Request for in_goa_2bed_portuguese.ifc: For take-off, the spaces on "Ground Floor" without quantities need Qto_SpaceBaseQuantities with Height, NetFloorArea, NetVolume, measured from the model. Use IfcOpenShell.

First a look at what the model holds.

```python
import ifcopenshell
import ifcopenshell.util.element
import ifcopenshell.util.unit

model = ifcopenshell.open("in_goa_2bed_portuguese.ifc")
print(model.schema)
for unit_type in ("LENGTHUNIT", "AREAUNIT", "VOLUMEUNIT"):
    print(unit_type, ifcopenshell.util.unit.calculate_unit_scale(model, unit_type))
storey = next(s for s in model.by_type("IfcBuildingStorey") if s.Name == "Ground Floor")
spaces = [e for e in ifcopenshell.util.element.get_decomposition(storey) if e.is_a("IfcSpace")]
for e in sorted(spaces, key=lambda e: e.id()):
    print(e.id(), e.is_a(), e.Name, list(ifcopenshell.util.element.get_psets(e, qtos_only=True)), sep=" | ")
```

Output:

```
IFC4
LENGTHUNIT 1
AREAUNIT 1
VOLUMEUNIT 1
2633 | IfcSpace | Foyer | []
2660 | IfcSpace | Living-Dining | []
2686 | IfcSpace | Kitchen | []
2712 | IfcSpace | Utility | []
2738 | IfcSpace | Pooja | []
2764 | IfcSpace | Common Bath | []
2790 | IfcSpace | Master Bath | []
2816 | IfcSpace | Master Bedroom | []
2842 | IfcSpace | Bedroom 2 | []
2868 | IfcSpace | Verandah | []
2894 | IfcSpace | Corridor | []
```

```python
import ifcopenshell
import ifcopenshell.api.pset
import ifcopenshell.geom
import ifcopenshell.util.element
import ifcopenshell.util.shape
import ifcopenshell.util.unit

model = ifcopenshell.open("in_goa_2bed_portuguese.ifc")
unit_scale = ifcopenshell.util.unit.calculate_unit_scale(model)
area_scale = ifcopenshell.util.unit.calculate_unit_scale(model, "AREAUNIT")
volume_scale = ifcopenshell.util.unit.calculate_unit_scale(model, "VOLUMEUNIT")
settings = ifcopenshell.geom.settings()

storey = next(s for s in model.by_type("IfcBuildingStorey") if s.Name == "Ground Floor")
spaces = [e for e in ifcopenshell.util.element.get_decomposition(storey) if e.is_a("IfcSpace")]

for e in sorted(spaces, key=lambda e: e.id()):
    if ifcopenshell.util.element.get_psets(e, qtos_only=True, should_inherit=False):
        continue
    # Geometry comes back in metres, in the element's own axes.
    shape = ifcopenshell.geom.create_shape(settings, e)
    values = {
        "Height": ifcopenshell.util.shape.get_z(shape.geometry) / unit_scale,
        "NetFloorArea": ifcopenshell.util.shape.get_footprint_area(shape.geometry) / area_scale,
        "NetVolume": ifcopenshell.util.shape.get_volume(shape.geometry) / volume_scale,
    }
    qto = ifcopenshell.api.pset.add_qto(model, product=e, name="Qto_SpaceBaseQuantities")
    ifcopenshell.api.pset.edit_qto(model, qto=qto, properties=values)
    print(e.id(), {k: round(v, 3) for k, v in values.items()})

model.write("in_goa_2bed_portuguese_edited.ifc")
```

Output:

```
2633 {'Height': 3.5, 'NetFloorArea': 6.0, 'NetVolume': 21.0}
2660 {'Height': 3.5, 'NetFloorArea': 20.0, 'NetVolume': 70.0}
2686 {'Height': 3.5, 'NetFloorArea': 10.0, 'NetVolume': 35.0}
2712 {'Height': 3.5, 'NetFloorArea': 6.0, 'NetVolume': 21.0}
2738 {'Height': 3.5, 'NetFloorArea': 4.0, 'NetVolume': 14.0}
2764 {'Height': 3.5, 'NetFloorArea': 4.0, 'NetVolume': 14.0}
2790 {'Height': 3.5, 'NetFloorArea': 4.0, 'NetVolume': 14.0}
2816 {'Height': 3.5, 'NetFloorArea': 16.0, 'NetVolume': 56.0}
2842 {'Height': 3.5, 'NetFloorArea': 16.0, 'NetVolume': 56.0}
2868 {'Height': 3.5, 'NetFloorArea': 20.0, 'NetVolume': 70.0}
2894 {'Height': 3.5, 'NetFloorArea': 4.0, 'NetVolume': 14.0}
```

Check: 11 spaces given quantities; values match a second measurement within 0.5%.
